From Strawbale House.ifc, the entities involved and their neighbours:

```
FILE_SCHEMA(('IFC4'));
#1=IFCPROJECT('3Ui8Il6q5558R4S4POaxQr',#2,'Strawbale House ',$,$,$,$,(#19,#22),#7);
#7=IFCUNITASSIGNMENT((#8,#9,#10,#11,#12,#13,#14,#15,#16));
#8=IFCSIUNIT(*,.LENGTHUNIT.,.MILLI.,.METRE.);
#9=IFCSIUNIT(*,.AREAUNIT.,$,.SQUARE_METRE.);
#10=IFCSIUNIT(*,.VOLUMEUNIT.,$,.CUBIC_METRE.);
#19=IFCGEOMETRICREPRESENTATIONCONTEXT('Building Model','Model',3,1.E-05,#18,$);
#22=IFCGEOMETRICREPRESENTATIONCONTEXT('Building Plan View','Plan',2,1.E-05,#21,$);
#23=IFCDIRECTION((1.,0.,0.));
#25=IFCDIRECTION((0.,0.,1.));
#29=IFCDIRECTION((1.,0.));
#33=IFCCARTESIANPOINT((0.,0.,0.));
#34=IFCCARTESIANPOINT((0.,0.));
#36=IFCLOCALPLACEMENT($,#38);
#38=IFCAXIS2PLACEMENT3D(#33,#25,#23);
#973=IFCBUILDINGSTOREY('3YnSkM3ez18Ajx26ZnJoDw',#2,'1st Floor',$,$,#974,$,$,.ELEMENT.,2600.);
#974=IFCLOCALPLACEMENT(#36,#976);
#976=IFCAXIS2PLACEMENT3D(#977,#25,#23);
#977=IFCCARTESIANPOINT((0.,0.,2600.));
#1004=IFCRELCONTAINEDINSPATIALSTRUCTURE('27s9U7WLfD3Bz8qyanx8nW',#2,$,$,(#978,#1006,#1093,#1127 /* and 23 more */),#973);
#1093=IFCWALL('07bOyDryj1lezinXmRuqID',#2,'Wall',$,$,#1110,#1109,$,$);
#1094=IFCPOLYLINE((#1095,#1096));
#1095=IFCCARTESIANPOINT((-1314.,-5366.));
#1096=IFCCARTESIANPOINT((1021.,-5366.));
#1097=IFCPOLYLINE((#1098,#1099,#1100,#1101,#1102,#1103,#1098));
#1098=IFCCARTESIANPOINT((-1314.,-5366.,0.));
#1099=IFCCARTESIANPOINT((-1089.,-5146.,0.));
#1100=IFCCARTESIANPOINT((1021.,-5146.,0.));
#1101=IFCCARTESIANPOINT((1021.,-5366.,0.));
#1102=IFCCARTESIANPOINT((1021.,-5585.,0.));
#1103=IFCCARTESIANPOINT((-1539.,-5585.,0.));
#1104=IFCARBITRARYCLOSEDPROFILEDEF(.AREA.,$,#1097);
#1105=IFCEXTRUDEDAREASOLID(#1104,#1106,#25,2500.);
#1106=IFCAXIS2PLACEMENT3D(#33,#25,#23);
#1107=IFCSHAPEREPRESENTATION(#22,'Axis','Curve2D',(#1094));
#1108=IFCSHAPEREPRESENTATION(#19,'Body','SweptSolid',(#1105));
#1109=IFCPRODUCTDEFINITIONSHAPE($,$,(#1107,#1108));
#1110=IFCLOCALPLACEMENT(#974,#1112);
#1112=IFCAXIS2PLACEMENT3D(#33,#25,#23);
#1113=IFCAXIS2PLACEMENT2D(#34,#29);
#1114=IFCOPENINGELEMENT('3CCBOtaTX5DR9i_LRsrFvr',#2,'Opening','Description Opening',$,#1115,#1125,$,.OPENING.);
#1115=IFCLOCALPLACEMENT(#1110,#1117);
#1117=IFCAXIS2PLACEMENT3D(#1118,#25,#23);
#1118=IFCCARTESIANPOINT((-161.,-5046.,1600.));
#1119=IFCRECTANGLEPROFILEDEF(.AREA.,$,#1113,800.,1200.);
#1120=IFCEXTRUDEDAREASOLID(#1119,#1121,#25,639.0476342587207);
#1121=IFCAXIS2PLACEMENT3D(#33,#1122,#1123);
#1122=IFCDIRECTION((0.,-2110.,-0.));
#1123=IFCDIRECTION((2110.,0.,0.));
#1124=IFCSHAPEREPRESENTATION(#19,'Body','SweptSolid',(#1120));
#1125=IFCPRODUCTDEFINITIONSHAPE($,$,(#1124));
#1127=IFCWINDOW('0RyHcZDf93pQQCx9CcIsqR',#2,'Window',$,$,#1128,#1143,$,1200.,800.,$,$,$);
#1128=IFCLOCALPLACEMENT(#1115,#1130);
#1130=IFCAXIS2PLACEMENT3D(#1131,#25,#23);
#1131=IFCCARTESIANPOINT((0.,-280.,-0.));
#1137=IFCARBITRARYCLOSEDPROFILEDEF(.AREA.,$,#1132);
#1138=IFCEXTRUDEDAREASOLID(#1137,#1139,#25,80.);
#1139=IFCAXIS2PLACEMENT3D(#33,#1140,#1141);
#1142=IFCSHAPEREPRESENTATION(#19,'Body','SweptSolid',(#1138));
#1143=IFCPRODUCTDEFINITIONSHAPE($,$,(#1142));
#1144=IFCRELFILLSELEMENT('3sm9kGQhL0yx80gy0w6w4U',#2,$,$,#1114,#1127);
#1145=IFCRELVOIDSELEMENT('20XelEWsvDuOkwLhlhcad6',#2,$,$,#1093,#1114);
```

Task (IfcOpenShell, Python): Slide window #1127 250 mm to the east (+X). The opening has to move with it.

```python
import ifcopenshell
import ifcopenshell.api.geometry
import ifcopenshell.util.placement
import ifcopenshell.util.unit

model = ifcopenshell.open("Strawbale House.ifc")
unit_scale = ifcopenshell.util.unit.calculate_unit_scale(model)

window = model.by_id(1127)
opening = window.FillsVoids[0].RelatingOpeningElement
wall = opening.VoidsElements[0].RelatingBuildingElement

wall_matrix = ifcopenshell.util.placement.get_local_placement(wall.ObjectPlacement)
shift = wall_matrix[:3, 0] * 0.25 / unit_scale
before = ifcopenshell.util.placement.get_local_placement(window.ObjectPlacement)[:3, 3].copy()

# The window is placed relative to its opening, so it follows when the opening moves.
matrix = ifcopenshell.util.placement.get_local_placement(opening.ObjectPlacement)
matrix[:3, 3] += shift
ifcopenshell.api.geometry.edit_object_placement(
    model, product=opening, matrix=matrix, is_si=False, should_transform_children=True
)

after = ifcopenshell.util.placement.get_local_placement(window.ObjectPlacement)[:3, 3]
print("window moved by", (after - before).round(3) + 0.0)

model.write("Strawbale House_edited.ifc")
```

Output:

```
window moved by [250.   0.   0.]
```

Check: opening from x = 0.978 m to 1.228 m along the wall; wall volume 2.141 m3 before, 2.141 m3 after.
